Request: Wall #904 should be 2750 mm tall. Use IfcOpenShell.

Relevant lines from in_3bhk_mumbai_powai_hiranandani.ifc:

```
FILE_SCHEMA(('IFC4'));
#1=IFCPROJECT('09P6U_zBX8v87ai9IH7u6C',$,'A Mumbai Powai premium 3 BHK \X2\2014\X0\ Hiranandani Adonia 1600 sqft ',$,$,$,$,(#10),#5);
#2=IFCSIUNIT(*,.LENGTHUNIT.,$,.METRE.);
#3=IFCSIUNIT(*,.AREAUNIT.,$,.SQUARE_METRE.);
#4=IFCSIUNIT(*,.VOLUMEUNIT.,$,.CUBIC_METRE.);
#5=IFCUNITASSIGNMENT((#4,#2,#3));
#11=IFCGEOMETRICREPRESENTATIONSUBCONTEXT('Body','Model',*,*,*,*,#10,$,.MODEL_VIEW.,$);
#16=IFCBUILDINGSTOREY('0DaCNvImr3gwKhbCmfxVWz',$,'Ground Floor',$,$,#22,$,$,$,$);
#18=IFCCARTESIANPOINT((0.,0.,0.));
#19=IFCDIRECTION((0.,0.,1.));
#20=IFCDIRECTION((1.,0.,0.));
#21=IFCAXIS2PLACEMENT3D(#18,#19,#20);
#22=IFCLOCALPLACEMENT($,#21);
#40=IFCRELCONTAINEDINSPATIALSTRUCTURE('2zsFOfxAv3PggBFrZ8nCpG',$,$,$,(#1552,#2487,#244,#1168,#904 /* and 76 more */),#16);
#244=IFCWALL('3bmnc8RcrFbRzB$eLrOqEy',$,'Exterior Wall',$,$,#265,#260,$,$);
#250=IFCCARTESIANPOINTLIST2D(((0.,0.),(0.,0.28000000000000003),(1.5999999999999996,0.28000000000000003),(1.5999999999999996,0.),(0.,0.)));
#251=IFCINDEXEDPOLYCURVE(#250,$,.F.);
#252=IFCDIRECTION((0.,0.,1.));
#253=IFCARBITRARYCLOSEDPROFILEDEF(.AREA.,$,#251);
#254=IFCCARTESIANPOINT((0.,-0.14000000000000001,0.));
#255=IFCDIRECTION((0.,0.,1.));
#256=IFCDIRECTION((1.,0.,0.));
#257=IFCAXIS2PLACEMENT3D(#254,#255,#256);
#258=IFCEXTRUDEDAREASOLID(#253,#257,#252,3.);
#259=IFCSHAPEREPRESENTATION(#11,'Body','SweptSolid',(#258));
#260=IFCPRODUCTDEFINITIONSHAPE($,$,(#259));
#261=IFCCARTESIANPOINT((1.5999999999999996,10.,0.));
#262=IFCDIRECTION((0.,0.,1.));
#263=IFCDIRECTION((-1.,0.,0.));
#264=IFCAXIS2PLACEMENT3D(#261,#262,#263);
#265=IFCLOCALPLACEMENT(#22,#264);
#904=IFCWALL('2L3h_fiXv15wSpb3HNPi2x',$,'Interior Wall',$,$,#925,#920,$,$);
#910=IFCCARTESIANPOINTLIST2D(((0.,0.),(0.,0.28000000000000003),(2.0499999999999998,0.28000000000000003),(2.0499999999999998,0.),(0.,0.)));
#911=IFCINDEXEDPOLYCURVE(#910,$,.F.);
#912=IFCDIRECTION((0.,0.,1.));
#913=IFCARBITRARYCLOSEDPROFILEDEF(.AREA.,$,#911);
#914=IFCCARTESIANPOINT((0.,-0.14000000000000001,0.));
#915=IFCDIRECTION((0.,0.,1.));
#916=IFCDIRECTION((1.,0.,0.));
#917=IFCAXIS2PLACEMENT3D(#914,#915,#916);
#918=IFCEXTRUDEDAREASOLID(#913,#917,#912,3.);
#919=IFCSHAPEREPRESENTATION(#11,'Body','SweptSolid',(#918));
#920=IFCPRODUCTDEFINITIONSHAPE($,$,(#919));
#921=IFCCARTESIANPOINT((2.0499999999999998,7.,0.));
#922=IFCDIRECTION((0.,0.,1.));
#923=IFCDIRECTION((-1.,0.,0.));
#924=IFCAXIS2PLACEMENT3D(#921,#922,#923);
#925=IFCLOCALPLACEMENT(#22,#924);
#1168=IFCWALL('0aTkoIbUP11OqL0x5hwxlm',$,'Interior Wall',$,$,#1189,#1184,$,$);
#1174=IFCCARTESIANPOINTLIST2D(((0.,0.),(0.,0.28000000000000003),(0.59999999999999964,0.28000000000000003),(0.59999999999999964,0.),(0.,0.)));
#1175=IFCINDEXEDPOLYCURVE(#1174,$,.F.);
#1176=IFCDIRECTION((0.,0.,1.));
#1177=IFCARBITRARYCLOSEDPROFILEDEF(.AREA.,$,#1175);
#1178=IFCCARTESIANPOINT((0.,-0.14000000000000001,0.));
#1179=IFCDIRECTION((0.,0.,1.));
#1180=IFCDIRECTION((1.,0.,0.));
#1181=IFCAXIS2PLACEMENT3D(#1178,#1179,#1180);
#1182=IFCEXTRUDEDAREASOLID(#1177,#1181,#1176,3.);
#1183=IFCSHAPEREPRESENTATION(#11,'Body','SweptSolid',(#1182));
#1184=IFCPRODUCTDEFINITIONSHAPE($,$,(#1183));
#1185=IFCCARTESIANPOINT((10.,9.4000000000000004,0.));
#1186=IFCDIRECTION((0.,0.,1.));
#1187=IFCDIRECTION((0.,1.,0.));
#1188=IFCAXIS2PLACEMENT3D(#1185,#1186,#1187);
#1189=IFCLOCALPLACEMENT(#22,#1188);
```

```python
import ifcopenshell
import ifcopenshell.geom
import ifcopenshell.util.representation
import ifcopenshell.util.shape
import ifcopenshell.util.unit

model = ifcopenshell.open("in_3bhk_mumbai_powai_hiranandani.ifc")
unit_scale = ifcopenshell.util.unit.calculate_unit_scale(model)
settings = ifcopenshell.geom.settings()


def volume(element):
    """Net volume in cubic metres, openings subtracted."""
    shape = ifcopenshell.geom.create_shape(settings, element)
    return ifcopenshell.util.shape.get_volume(shape.geometry)


wall = model.by_id(904)
before = volume(wall)

body = ifcopenshell.util.representation.get_representation(wall, "Model", "Body")
solid = body.Items[0]
old_height = solid.Depth
solid.Depth = 2.75 / unit_scale
after = volume(wall)

print(f"height {old_height:g} -> {solid.Depth:g}, volume {before:.3f} -> {after:.3f} m3")

model.write("in_3bhk_mumbai_powai_hiranandani-out.ifc")
```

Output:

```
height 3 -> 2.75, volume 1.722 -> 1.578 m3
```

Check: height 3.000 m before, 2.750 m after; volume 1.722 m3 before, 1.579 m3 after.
